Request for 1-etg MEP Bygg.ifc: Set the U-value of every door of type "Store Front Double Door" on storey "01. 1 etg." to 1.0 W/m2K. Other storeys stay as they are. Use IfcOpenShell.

First a look at what the model holds.

```python
import ifcopenshell
import ifcopenshell.util.element

model = ifcopenshell.open("1-etg MEP Bygg.ifc")
print(model.schema)
storey = next(s for s in model.by_type("IfcBuildingStorey") if s.Name == "01. 1 etg.")
doors = [e for e in ifcopenshell.util.element.get_decomposition(storey) if e.is_a("IfcDoor")]
seen = {}
for e in doors:
    element_type = ifcopenshell.util.element.get_type(e)
    key = (element_type.Name if element_type != e and element_type else None, ifcopenshell.util.element.get_pset(e, "Pset_DoorCommon", "ThermalTransmittance"))
    seen[key] = seen.get(key, 0) + 1
for (name, value), count in sorted(seen.items(), key=str):
    print(count, "x", name, "|", value)
```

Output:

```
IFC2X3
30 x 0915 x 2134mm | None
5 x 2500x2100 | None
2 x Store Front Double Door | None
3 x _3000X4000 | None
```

```python
import ifcopenshell
import ifcopenshell.api.pset
import ifcopenshell.util.element

model = ifcopenshell.open("1-etg MEP Bygg.ifc")

storey = next(s for s in model.by_type("IfcBuildingStorey") if s.Name == "01. 1 etg.")
doors = [e for e in ifcopenshell.util.element.get_decomposition(storey) if e.is_a("IfcDoor")]

count = 0
for e in doors:
    element_type = ifcopenshell.util.element.get_type(e)
    if element_type in (None, e) or element_type.Name != "Store Front Double Door":
        continue
    # add_pset returns the element's existing set when there is one.
    pset = ifcopenshell.api.pset.add_pset(model, product=e, name="Pset_DoorCommon")
    ifcopenshell.api.pset.edit_pset(model, pset=pset, properties={"ThermalTransmittance": 1.0})
    count += 1

print(count, "doors updated")

model.write("1-etg MEP Bygg_updated.ifc")
```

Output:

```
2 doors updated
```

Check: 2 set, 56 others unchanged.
